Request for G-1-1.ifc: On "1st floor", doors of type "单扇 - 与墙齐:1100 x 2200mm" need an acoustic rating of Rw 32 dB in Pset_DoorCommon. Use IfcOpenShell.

First a look at what the model holds.

```python
import ifcopenshell
import ifcopenshell.util.element

model = ifcopenshell.open("G-1-1.ifc")
print(model.schema)
storey = next(s for s in model.by_type("IfcBuildingStorey") if s.Name == "1st floor")
doors = [e for e in ifcopenshell.util.element.get_decomposition(storey) if e.is_a("IfcDoor")]
seen = {}
for e in doors:
    element_type = ifcopenshell.util.element.get_type(e)
    key = (element_type.Name if element_type != e and element_type else None, ifcopenshell.util.element.get_pset(e, "Pset_DoorCommon", "AcousticRating"))
    seen[key] = seen.get(key, 0) + 1
for (name, value), count in sorted(seen.items(), key=str):
    print(count, "x", name, "|", value)
```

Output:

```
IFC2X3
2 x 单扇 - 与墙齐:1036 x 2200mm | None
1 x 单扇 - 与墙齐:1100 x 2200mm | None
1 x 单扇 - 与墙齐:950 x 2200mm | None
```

```python
import ifcopenshell
import ifcopenshell.api.pset
import ifcopenshell.util.element

model = ifcopenshell.open("G-1-1.ifc")

storey = next(s for s in model.by_type("IfcBuildingStorey") if s.Name == "1st floor")
doors = [e for e in ifcopenshell.util.element.get_decomposition(storey) if e.is_a("IfcDoor")]

count = 0
for e in doors:
    element_type = ifcopenshell.util.element.get_type(e)
    if element_type in (None, e) or element_type.Name != "单扇 - 与墙齐:1100 x 2200mm":
        continue
    # add_pset returns the element's existing set when there is one.
    pset = ifcopenshell.api.pset.add_pset(model, product=e, name="Pset_DoorCommon")
    ifcopenshell.api.pset.edit_pset(model, pset=pset, properties={"AcousticRating": "Rw 32 dB"})
    count += 1

print(count, "doors updated")

model.write("G-1-1_updated.ifc")
```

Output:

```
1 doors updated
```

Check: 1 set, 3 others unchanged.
